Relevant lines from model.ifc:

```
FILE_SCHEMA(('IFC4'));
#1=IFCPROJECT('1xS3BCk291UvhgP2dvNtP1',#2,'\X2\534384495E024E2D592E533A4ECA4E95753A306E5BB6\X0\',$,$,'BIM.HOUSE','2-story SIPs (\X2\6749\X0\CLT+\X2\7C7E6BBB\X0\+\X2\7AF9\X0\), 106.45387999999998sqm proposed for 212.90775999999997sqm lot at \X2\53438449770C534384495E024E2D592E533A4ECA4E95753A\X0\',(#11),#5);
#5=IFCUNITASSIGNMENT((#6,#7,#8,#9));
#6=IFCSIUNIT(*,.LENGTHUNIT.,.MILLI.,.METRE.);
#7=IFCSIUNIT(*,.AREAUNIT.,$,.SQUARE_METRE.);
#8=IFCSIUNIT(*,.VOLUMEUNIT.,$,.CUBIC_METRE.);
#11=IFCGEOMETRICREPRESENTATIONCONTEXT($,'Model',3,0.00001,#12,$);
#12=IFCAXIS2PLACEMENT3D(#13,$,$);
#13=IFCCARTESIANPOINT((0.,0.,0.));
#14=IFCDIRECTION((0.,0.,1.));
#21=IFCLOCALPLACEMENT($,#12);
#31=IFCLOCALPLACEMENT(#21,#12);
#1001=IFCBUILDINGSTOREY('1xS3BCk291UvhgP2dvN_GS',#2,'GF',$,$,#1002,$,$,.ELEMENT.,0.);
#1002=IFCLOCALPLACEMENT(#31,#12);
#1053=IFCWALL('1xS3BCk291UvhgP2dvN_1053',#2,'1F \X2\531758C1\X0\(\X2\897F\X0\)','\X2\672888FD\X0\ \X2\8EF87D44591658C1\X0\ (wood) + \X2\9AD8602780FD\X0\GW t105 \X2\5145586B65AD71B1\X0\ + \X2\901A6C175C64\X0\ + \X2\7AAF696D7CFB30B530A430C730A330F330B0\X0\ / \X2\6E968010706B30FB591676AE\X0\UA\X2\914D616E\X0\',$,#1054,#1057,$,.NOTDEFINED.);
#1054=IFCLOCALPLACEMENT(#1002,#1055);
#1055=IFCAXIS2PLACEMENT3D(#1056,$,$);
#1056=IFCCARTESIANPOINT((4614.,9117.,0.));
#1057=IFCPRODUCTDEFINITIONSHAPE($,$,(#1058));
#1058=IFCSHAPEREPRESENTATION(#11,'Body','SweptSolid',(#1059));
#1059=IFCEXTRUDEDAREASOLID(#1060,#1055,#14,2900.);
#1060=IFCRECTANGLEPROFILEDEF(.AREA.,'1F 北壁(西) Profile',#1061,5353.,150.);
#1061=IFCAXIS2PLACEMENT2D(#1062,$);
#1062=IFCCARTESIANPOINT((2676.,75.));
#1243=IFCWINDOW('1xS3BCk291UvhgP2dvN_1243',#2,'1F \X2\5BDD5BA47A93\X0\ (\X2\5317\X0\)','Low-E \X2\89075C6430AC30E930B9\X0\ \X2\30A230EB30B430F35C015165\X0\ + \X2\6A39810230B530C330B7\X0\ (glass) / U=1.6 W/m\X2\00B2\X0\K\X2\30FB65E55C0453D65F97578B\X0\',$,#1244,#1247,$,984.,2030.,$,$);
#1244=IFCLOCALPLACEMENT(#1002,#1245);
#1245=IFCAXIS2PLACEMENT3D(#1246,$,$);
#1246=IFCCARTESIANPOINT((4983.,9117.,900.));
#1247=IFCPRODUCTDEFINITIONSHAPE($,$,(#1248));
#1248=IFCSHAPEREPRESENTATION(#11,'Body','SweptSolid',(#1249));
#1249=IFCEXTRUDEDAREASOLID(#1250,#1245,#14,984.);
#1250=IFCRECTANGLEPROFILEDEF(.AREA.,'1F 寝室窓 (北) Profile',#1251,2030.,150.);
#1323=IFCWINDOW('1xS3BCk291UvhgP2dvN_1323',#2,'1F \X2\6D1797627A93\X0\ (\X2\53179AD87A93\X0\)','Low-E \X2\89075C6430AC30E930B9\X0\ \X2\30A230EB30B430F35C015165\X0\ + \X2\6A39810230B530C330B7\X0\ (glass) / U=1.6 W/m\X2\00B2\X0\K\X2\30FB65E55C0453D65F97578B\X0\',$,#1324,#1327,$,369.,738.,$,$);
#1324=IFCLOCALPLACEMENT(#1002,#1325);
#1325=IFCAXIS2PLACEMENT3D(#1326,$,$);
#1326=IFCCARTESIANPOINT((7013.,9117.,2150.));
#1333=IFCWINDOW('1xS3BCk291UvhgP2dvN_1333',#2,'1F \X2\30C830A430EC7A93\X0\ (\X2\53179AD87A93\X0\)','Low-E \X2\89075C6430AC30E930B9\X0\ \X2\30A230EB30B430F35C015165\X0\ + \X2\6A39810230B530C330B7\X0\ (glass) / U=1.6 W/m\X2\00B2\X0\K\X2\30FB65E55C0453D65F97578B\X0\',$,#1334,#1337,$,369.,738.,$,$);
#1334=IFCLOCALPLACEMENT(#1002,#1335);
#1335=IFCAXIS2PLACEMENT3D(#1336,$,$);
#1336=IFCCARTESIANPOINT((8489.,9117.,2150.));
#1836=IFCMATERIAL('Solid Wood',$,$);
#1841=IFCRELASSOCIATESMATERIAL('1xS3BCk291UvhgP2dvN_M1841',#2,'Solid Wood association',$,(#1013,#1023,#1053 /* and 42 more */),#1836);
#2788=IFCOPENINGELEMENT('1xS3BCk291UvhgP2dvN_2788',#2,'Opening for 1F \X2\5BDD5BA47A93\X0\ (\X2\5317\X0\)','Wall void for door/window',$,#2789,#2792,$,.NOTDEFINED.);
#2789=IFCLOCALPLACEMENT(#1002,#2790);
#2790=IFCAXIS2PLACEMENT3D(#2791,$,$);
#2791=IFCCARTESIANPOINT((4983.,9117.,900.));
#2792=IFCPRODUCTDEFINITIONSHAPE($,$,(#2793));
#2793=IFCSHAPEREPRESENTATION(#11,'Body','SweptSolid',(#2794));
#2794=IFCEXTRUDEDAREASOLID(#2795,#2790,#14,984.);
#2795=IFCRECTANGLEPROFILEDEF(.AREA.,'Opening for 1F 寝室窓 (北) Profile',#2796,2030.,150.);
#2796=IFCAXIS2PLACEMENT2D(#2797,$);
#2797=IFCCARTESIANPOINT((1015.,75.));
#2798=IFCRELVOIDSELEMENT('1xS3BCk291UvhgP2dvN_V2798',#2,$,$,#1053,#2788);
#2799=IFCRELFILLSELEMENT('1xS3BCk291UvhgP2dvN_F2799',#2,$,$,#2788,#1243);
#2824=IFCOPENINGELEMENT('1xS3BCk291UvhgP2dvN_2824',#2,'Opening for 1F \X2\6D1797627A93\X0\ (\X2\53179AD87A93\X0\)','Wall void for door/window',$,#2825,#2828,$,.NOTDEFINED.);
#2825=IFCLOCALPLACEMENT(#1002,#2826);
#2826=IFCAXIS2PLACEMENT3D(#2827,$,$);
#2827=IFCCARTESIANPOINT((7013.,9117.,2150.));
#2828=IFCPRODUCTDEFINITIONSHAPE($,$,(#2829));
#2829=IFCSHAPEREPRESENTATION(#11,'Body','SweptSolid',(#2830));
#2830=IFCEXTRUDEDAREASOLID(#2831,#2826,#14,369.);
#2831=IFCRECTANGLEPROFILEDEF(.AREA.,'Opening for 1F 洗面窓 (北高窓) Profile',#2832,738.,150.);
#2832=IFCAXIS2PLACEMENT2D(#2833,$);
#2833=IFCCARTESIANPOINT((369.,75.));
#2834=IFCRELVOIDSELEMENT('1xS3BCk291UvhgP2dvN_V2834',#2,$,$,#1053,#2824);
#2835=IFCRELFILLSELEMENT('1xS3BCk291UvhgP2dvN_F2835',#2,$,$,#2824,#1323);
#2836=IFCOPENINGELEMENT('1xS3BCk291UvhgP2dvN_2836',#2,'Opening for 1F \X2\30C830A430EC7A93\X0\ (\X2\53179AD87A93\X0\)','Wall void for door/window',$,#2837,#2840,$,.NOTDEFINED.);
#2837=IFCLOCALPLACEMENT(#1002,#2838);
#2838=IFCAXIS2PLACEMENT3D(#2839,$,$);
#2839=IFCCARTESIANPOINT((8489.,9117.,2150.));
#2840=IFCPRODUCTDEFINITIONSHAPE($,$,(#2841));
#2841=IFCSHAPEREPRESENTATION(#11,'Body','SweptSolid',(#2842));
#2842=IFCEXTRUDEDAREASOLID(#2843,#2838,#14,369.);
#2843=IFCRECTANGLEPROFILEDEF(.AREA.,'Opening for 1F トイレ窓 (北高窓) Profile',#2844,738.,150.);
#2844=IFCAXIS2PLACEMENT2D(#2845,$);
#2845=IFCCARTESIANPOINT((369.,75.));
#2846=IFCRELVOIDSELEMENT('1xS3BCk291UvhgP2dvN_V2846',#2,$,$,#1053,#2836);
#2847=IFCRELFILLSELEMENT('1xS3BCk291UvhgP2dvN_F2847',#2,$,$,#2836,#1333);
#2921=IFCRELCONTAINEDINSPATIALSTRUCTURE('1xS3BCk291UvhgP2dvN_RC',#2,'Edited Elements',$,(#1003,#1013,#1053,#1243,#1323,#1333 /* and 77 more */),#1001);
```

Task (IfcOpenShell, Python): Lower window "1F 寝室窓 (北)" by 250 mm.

```python
import numpy as np
import ifcopenshell
import ifcopenshell.api.geometry
import ifcopenshell.util.placement
import ifcopenshell.util.unit

model = ifcopenshell.open("model.ifc")
unit_scale = ifcopenshell.util.unit.calculate_unit_scale(model)

window = model.by_guid("1xS3BCk291UvhgP2dvN_1243")
opening = window.FillsVoids[0].RelatingOpeningElement
dz = -250.0

shift = np.array([0.0, 0.0, dz])
# The window is not placed relative to its opening, so move both.
for product in (opening, window):
    matrix = ifcopenshell.util.placement.get_local_placement(product.ObjectPlacement)
    matrix[:3, 3] += shift
    ifcopenshell.api.geometry.edit_object_placement(model, product=product, matrix=matrix, is_si=False)

print(f"moved by {dz * unit_scale:+.3f} m")

model.write("model_updated.ifc")
```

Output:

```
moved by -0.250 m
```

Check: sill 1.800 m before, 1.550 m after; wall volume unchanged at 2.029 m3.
